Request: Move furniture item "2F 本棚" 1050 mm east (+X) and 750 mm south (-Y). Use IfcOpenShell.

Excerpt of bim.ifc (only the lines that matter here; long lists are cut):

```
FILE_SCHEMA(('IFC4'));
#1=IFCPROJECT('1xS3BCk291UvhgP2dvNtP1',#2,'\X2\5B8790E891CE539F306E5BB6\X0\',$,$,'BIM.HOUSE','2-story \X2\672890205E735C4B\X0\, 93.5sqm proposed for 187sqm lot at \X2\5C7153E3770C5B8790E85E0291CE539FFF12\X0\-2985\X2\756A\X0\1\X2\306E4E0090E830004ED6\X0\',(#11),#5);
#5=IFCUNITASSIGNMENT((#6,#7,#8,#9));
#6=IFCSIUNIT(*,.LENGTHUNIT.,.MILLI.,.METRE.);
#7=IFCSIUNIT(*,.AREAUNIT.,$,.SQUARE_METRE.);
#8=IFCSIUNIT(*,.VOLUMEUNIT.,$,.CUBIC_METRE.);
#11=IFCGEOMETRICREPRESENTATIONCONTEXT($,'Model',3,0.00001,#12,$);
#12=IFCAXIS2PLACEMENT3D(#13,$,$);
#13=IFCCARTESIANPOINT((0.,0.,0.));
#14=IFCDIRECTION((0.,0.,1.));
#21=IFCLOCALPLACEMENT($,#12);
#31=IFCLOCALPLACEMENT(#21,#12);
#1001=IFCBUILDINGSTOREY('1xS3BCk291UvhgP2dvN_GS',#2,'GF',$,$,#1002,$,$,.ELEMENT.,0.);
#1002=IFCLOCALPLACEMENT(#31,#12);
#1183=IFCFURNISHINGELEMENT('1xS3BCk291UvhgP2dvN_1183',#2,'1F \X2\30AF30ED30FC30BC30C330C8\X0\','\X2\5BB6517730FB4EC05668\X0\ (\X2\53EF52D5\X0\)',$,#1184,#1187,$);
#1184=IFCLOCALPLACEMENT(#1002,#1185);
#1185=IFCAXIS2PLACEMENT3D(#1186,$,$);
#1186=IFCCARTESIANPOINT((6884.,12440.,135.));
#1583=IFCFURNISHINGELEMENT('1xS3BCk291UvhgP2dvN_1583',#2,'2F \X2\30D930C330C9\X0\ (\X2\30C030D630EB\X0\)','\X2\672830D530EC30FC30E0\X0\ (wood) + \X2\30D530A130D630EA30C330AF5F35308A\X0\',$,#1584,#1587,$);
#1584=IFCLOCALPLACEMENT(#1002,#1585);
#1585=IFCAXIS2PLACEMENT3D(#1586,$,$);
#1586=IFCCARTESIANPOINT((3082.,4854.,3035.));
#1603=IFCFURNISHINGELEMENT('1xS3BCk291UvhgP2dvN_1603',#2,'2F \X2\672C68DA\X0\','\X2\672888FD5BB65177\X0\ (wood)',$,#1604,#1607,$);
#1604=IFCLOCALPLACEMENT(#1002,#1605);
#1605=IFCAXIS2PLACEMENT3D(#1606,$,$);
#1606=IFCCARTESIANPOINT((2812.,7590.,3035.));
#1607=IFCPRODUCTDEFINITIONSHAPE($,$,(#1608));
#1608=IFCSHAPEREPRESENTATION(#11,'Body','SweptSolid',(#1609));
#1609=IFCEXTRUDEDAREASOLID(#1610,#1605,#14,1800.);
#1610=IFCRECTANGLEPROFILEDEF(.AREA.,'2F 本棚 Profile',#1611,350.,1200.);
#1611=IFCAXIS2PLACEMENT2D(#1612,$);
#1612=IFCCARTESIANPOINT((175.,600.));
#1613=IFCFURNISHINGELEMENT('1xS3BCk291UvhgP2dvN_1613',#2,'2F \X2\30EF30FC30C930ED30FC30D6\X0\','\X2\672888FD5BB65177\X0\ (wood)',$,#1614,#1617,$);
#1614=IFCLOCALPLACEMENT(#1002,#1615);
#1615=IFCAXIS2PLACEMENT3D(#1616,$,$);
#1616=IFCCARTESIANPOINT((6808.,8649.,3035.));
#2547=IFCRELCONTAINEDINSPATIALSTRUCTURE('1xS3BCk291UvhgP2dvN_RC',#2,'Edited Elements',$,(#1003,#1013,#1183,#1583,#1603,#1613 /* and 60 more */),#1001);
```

```python
import ifcopenshell
import ifcopenshell.api.geometry
import ifcopenshell.util.placement

model = ifcopenshell.open("bim.ifc")

item = model.by_guid("1xS3BCk291UvhgP2dvN_1603")
matrix = ifcopenshell.util.placement.get_local_placement(item.ObjectPlacement)
matrix[0, 3] += 1050.0
matrix[1, 3] -= 750.0
ifcopenshell.api.geometry.edit_object_placement(model, product=item, matrix=matrix, is_si=False)

print(ifcopenshell.util.placement.get_local_placement(item.ObjectPlacement).round(3) + 0.0)

model.write("bim_v2.ifc")
```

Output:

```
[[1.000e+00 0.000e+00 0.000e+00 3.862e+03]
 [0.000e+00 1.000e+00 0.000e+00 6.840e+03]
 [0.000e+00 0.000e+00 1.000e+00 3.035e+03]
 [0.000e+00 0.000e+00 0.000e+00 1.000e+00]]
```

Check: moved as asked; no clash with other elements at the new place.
